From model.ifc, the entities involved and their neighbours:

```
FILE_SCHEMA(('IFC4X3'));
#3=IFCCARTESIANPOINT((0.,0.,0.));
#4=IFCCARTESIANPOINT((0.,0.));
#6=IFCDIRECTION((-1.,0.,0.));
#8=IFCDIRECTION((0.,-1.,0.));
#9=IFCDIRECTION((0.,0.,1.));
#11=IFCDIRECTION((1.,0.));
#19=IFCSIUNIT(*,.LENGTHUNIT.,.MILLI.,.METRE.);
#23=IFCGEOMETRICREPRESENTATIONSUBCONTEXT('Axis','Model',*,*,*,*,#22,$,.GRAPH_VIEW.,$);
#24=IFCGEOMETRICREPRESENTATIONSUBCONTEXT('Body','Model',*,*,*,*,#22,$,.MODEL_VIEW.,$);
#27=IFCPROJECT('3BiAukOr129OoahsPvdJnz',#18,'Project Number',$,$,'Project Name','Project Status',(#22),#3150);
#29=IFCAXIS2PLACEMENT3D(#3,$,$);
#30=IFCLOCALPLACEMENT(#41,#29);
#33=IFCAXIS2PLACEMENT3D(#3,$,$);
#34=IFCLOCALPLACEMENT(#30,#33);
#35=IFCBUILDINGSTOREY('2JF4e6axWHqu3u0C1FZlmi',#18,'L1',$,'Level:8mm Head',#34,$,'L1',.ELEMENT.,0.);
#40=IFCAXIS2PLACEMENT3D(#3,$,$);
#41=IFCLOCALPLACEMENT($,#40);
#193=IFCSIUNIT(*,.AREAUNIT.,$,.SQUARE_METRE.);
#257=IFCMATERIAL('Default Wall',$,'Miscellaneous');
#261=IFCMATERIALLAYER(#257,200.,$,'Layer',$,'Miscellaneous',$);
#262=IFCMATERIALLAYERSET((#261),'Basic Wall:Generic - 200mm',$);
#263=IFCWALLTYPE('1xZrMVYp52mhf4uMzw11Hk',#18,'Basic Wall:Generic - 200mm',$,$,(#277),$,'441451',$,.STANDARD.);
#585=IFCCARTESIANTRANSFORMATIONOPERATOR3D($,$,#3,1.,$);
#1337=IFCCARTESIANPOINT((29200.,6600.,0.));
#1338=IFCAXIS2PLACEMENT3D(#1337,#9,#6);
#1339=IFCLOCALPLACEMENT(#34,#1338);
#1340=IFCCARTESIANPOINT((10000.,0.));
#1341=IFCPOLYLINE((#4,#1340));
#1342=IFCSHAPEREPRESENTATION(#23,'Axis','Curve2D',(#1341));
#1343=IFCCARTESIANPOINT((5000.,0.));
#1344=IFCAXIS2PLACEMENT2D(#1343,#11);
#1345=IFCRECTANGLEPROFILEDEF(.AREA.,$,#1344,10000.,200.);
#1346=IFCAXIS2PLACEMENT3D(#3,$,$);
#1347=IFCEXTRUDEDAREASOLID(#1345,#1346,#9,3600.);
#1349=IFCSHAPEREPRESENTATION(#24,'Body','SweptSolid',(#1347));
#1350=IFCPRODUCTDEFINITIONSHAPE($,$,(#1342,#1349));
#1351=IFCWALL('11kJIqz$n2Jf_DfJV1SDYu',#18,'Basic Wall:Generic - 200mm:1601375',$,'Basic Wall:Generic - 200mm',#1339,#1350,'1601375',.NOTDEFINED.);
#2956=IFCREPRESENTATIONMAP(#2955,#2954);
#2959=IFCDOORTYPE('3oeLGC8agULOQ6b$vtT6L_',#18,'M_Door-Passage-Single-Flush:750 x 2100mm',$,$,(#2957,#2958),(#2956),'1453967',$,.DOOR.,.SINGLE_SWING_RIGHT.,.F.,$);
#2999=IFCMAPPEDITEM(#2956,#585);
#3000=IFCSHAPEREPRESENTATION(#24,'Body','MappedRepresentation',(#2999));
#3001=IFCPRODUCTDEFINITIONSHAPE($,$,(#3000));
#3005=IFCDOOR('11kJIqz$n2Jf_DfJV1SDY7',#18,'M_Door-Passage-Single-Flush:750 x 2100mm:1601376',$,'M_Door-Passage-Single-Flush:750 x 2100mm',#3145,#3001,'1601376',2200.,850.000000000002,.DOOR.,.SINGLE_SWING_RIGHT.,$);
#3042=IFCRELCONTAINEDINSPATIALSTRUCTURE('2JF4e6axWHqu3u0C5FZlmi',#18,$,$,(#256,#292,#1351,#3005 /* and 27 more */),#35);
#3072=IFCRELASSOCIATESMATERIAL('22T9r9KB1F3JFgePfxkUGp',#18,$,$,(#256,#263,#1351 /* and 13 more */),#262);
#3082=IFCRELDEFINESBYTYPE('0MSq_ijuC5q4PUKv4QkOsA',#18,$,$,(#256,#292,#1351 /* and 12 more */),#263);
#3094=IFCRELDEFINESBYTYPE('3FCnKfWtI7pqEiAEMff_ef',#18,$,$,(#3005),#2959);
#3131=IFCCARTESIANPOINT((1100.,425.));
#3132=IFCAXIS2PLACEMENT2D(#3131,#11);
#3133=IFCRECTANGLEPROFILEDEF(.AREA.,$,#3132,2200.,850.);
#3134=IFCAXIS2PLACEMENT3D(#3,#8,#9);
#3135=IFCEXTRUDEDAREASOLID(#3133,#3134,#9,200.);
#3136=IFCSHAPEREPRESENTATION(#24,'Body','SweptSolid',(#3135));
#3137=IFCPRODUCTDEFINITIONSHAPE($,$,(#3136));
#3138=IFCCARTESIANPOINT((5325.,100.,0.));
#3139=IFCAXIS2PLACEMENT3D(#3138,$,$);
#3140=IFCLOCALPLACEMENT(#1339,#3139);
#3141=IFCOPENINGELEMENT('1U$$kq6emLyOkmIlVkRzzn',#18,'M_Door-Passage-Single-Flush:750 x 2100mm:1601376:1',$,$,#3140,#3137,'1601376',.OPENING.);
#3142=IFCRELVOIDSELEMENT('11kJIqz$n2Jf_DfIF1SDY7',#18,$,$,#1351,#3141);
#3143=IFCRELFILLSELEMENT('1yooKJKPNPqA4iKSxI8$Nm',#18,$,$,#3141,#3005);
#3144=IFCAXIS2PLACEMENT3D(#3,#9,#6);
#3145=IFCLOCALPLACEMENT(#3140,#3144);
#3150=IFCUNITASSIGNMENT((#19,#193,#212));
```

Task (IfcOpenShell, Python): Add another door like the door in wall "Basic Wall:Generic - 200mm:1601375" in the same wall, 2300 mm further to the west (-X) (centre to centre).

```python
import ifcopenshell
import ifcopenshell.api.feature
import ifcopenshell.api.geometry
import ifcopenshell.api.root
import ifcopenshell.geom
import ifcopenshell.util.element
import ifcopenshell.util.placement
import ifcopenshell.util.shape
import ifcopenshell.util.unit

model = ifcopenshell.open("model.ifc")
unit_scale = ifcopenshell.util.unit.calculate_unit_scale(model)
settings = ifcopenshell.geom.settings()


def volume(element):
    """Net volume in cubic metres, openings subtracted."""
    shape = ifcopenshell.geom.create_shape(settings, element)
    return ifcopenshell.util.shape.get_volume(shape.geometry)


def reuse_history(source, copy):
    """copy_class also copies each property set's owner history, people and application; keep the originals."""
    for rel in copy.IsDefinedBy:
        if rel.is_a("IfcRelDefinesByProperties") and (history := rel.RelatingPropertyDefinition.OwnerHistory):
            rel.RelatingPropertyDefinition.OwnerHistory = source.OwnerHistory
            ifcopenshell.util.element.remove_deep2(model, history)


door = model.by_guid("11kJIqz$n2Jf_DfJV1SDY7")
opening = door.FillsVoids[0].RelatingOpeningElement
wall = opening.VoidsElements[0].RelatingBuildingElement
before = volume(wall)
shift = ifcopenshell.util.placement.get_local_placement(wall.ObjectPlacement)[:3, 0] * 2.3 / unit_scale

# copy_class copies the void relationship, type, container and properties, but no geometry.
new_opening = ifcopenshell.api.root.copy_class(model, product=opening)
new_opening.Representation = ifcopenshell.util.element.copy_deep(
    model, opening.Representation, exclude=["IfcGeometricRepresentationContext", "IfcRepresentationMap"]
)
new_opening.Name = "M_Door-Passage-Single-Flush:750 x 2100mm"
new_opening.Tag = None
new_door = ifcopenshell.api.root.copy_class(model, product=door)
new_door.Representation = ifcopenshell.util.element.copy_deep(
    model, door.Representation, exclude=["IfcGeometricRepresentationContext", "IfcRepresentationMap"]
)
new_door.Name = "M_Door-Passage-Single-Flush:750 x 2100mm"
new_door.Tag = None
reuse_history(door, new_door)
ifcopenshell.api.feature.add_filling(model, opening=new_opening, element=new_door)

for old, new in ((opening, new_opening), (door, new_door)):
    matrix = ifcopenshell.util.placement.get_local_placement(old.ObjectPlacement)
    matrix[:3, 3] += shift
    ifcopenshell.api.geometry.edit_object_placement(model, product=new, matrix=matrix, is_si=False)

after = volume(wall)

print(f"wall volume {before:.3f} -> {after:.3f} m3")

model.write("model_v2.ifc")
```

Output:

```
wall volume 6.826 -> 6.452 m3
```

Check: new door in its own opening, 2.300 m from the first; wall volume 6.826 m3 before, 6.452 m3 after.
